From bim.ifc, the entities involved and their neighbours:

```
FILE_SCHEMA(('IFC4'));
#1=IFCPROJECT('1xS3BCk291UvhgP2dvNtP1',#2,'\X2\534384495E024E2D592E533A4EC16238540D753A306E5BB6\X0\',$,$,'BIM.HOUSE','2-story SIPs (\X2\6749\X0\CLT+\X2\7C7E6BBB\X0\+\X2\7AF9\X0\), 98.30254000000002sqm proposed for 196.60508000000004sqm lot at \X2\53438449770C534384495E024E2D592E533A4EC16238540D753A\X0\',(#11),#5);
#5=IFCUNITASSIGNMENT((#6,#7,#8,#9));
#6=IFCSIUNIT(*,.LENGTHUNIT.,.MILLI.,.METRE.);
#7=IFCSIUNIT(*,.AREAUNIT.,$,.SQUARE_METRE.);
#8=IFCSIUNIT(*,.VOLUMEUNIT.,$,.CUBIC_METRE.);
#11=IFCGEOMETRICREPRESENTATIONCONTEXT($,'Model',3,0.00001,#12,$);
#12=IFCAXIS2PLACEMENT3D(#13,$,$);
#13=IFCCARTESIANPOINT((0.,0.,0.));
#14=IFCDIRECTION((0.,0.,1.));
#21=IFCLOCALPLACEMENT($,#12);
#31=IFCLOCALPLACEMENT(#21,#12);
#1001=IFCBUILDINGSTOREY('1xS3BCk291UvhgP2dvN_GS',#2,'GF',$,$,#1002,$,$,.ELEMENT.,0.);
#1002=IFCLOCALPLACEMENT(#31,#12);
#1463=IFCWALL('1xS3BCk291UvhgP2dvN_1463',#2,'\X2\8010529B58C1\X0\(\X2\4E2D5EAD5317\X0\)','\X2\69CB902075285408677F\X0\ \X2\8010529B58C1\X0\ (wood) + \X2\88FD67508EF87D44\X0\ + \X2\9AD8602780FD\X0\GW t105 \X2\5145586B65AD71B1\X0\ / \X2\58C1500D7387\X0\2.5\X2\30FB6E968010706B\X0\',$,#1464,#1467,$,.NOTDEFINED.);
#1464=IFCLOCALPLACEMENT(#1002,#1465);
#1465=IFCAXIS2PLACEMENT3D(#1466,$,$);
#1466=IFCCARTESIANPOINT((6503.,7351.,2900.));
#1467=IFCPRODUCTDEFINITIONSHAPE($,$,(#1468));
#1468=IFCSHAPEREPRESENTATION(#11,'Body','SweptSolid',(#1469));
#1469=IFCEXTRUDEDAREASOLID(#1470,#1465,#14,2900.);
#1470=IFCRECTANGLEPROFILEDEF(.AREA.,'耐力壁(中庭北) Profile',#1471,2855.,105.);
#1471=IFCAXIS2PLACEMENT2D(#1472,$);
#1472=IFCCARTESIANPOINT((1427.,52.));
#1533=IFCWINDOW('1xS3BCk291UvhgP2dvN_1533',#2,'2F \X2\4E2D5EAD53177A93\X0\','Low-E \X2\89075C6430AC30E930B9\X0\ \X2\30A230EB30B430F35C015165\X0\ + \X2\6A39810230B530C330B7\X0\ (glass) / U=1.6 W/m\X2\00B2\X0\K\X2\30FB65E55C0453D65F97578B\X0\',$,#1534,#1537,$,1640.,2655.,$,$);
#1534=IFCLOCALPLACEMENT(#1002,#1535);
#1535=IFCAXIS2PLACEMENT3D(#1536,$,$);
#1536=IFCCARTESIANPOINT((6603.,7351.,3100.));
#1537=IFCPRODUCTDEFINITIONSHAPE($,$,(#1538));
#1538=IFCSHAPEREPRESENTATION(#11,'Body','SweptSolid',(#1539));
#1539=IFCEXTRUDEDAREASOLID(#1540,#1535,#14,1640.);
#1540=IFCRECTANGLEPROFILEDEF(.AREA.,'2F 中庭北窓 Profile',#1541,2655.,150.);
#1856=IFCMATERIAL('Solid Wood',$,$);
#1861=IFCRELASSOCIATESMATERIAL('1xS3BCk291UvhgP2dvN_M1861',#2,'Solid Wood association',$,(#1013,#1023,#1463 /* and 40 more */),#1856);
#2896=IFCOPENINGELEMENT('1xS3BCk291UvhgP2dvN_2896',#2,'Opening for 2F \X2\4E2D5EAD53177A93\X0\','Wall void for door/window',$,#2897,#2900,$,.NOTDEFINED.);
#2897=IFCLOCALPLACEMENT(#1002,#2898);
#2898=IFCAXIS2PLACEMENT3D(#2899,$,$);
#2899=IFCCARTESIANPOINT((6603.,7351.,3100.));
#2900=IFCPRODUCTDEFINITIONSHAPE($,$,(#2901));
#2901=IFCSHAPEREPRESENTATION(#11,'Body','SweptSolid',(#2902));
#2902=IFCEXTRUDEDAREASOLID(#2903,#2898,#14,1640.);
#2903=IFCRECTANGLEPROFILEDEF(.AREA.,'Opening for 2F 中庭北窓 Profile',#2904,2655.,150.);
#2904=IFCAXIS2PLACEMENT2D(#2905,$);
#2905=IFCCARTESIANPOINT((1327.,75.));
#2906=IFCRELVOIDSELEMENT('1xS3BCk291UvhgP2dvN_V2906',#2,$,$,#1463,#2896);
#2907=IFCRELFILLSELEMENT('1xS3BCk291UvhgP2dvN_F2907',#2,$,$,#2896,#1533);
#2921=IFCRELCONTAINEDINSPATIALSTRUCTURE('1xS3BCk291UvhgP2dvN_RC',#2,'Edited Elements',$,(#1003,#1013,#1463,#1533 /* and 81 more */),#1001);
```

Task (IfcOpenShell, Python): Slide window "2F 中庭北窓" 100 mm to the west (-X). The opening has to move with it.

```python
import ifcopenshell
import ifcopenshell.api.geometry
import ifcopenshell.util.placement

model = ifcopenshell.open("bim.ifc")

window = model.by_guid("1xS3BCk291UvhgP2dvN_1533")
opening = window.FillsVoids[0].RelatingOpeningElement
wall = opening.VoidsElements[0].RelatingBuildingElement

wall_matrix = ifcopenshell.util.placement.get_local_placement(wall.ObjectPlacement)
shift = wall_matrix[:3, 0] * -100.0
before = ifcopenshell.util.placement.get_local_placement(window.ObjectPlacement)[:3, 3].copy()

# The window is not placed relative to its opening, so move both.
for product in (opening, window):
    matrix = ifcopenshell.util.placement.get_local_placement(product.ObjectPlacement)
    matrix[:3, 3] += shift
    ifcopenshell.api.geometry.edit_object_placement(model, product=product, matrix=matrix, is_si=False)

after = ifcopenshell.util.placement.get_local_placement(window.ObjectPlacement)[:3, 3]
print("window moved by", (after - before).round(3) + 0.0)

model.write("bim_rev.ifc")
```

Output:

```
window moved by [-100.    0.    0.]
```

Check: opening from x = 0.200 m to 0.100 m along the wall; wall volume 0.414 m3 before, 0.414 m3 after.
